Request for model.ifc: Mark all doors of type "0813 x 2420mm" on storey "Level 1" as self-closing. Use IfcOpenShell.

First a look at what the model holds.

```python
import ifcopenshell
import ifcopenshell.util.element

model = ifcopenshell.open("model.ifc")
print(model.schema)
storey = next(s for s in model.by_type("IfcBuildingStorey") if s.Name == "Level 1")
doors = [e for e in ifcopenshell.util.element.get_decomposition(storey) if e.is_a("IfcDoor")]
seen = {}
for e in doors:
    element_type = ifcopenshell.util.element.get_type(e)
    key = (element_type.Name if element_type != e and element_type else None, ifcopenshell.util.element.get_pset(e, "Pset_DoorCommon", "SelfClosing"))
    seen[key] = seen.get(key, 0) + 1
for (name, value), count in sorted(seen.items(), key=str):
    print(count, "x", name, "|", value)
```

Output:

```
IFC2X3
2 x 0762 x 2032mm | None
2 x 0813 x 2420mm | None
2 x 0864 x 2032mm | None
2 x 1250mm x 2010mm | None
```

```python
import ifcopenshell
import ifcopenshell.api.pset
import ifcopenshell.util.element

model = ifcopenshell.open("model.ifc")

storey = next(s for s in model.by_type("IfcBuildingStorey") if s.Name == "Level 1")
doors = [e for e in ifcopenshell.util.element.get_decomposition(storey) if e.is_a("IfcDoor")]

count = 0
for e in doors:
    element_type = ifcopenshell.util.element.get_type(e)
    if element_type in (None, e) or element_type.Name != "0813 x 2420mm":
        continue
    # add_pset returns the element's existing set when there is one.
    pset = ifcopenshell.api.pset.add_pset(model, product=e, name="Pset_DoorCommon")
    ifcopenshell.api.pset.edit_pset(model, pset=pset, properties={"SelfClosing": True})
    count += 1

print(count, "doors updated")

model.write("model_updated.ifc")
```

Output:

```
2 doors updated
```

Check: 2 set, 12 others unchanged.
